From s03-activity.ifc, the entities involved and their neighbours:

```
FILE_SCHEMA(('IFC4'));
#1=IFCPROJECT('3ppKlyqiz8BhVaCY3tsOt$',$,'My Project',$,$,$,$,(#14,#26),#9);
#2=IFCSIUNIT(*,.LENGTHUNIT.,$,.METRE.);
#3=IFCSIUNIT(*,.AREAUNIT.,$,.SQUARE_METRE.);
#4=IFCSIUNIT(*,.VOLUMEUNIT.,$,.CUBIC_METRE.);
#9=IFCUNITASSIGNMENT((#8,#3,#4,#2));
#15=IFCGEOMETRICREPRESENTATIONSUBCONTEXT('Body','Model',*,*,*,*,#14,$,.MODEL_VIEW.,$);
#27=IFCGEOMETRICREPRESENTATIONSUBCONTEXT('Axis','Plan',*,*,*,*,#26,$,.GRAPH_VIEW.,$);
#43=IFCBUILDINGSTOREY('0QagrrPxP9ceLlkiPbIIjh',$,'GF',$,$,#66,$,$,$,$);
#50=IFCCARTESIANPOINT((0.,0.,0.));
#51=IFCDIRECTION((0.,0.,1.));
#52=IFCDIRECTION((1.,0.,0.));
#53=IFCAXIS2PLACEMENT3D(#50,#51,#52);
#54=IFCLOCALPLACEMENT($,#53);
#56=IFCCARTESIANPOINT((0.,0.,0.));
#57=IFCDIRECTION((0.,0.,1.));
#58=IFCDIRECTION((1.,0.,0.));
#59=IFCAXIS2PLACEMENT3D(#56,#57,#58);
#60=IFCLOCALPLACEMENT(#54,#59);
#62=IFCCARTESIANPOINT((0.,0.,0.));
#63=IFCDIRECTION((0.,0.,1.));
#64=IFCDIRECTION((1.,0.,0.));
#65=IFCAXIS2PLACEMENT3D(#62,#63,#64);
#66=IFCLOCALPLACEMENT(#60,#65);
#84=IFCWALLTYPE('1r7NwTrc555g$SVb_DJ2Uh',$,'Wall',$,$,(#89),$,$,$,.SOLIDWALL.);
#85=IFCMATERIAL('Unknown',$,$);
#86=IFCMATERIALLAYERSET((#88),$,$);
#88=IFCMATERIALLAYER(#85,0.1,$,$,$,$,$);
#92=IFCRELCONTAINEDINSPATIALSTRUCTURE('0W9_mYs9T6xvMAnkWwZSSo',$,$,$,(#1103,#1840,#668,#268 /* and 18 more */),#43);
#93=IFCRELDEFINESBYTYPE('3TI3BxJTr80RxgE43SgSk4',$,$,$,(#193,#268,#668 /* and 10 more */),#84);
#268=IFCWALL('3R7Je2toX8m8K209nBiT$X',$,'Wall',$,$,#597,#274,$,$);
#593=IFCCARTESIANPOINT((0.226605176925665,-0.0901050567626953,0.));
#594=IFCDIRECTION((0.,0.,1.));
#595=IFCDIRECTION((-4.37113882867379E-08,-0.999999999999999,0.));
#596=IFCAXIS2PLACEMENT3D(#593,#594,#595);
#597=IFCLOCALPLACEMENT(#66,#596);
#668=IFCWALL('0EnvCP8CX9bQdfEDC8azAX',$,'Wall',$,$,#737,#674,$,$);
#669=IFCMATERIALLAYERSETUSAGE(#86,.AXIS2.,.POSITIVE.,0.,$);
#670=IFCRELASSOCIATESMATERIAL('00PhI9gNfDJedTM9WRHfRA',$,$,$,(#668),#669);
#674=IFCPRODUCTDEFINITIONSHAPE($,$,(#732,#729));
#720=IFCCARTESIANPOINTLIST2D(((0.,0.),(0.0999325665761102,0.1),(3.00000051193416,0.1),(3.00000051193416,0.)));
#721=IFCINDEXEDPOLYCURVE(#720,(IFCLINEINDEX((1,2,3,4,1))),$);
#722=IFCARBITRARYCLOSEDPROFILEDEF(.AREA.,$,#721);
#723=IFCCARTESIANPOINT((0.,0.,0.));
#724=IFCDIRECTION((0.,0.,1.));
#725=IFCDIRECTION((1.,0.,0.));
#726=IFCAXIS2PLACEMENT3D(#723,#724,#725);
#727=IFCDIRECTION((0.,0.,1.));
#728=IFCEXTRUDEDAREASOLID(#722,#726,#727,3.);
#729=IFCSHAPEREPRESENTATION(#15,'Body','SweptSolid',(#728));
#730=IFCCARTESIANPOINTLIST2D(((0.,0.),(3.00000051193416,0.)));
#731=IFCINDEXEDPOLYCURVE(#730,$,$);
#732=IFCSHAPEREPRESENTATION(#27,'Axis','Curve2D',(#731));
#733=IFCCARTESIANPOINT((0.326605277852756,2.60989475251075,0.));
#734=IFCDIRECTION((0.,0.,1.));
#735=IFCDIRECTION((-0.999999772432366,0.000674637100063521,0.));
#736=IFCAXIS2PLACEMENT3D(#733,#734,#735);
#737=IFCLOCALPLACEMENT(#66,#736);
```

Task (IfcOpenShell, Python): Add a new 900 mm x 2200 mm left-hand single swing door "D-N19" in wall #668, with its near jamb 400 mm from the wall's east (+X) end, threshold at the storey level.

```python
import numpy as np
import ifcopenshell
import ifcopenshell.api.feature
import ifcopenshell.api.geometry
import ifcopenshell.api.root
import ifcopenshell.api.spatial
import ifcopenshell.geom
import ifcopenshell.util.element
import ifcopenshell.util.placement
import ifcopenshell.util.representation
import ifcopenshell.util.shape
import ifcopenshell.util.unit

model = ifcopenshell.open("s03-activity.ifc")
unit_scale = ifcopenshell.util.unit.calculate_unit_scale(model)
settings = ifcopenshell.geom.settings()


def volume(element):
    """Net volume in cubic metres, openings subtracted."""
    shape = ifcopenshell.geom.create_shape(settings, element)
    return ifcopenshell.util.shape.get_volume(shape.geometry)


wall = model.by_guid("0EnvCP8CX9bQdfEDC8azAX")
storey = ifcopenshell.util.element.get_container(wall, ifc_class="IfcBuildingStorey")
context = ifcopenshell.util.representation.get_context(model, "Model", "Body", "MODEL_VIEW")
before = volume(wall)

width, height, from_end, sill = 0.9, 2.2, 0.4, 0.0  # metres

# The wall runs along its own X axis, and the end named is its -X end.
wall_shape = ifcopenshell.geom.create_shape(settings, wall)
x, y, z = ifcopenshell.util.shape.get_vertices(wall_shape.geometry).T
start = x.min() + from_end
face, thickness = float(y.min()), float(y.max() - y.min())
wall_matrix = ifcopenshell.util.placement.get_local_placement(wall.ObjectPlacement)
level = ifcopenshell.util.placement.get_local_placement(storey.ObjectPlacement)[2, 3]


def in_wall(x, y):
    """Placement at x, y metres in the wall's axes, at sill height."""
    matrix = wall_matrix.copy()
    matrix[:, 3] = wall_matrix @ np.array([x / unit_scale, y / unit_scale, 0.0, 1.0])
    matrix[2, 3] = level + sill / unit_scale
    return matrix


# Opening: a box that overshoots both wall faces by 50 mm.
opening = ifcopenshell.api.root.create_entity(model, ifc_class="IfcOpeningElement", predefined_type="OPENING")
box = ifcopenshell.api.geometry.add_wall_representation(
    model, context=context, length=width, height=height, thickness=thickness + 0.1
)
ifcopenshell.api.geometry.assign_representation(model, product=opening, representation=box)
ifcopenshell.api.geometry.edit_object_placement(model, product=opening, matrix=in_wall(start, face - 0.05), is_si=False)
ifcopenshell.api.feature.add_feature(model, feature=opening, element=wall)

door = ifcopenshell.api.root.create_entity(model, ifc_class="IfcDoor", name="D-N19", predefined_type="DOOR")
door.OverallWidth, door.OverallHeight = width / unit_scale, height / unit_scale
door.OperationType = "SINGLE_SWING_LEFT"
body = ifcopenshell.api.geometry.add_door_representation(
    model,
    context=context,
    overall_width=door.OverallWidth,
    overall_height=door.OverallHeight,
    operation_type="SINGLE_SWING_LEFT",
    lining_properties={"LiningDepth": thickness / unit_scale, "ThresholdDepth": thickness / unit_scale},
)
ifcopenshell.api.geometry.assign_representation(model, product=door, representation=body)
ifcopenshell.api.spatial.assign_container(model, products=[door], relating_structure=storey)
ifcopenshell.api.feature.add_filling(model, opening=opening, element=door)

# The lining spans the wall, so the door starts at the wall face.
ifcopenshell.api.geometry.edit_object_placement(model, product=door, matrix=in_wall(start, face), is_si=False)

after = volume(wall)

print(f"wall volume {before:.3f} -> {after:.3f} m3")

model.write("s03-activity_v2.ifc")
```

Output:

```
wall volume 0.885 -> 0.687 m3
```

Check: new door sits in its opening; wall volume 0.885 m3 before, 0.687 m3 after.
